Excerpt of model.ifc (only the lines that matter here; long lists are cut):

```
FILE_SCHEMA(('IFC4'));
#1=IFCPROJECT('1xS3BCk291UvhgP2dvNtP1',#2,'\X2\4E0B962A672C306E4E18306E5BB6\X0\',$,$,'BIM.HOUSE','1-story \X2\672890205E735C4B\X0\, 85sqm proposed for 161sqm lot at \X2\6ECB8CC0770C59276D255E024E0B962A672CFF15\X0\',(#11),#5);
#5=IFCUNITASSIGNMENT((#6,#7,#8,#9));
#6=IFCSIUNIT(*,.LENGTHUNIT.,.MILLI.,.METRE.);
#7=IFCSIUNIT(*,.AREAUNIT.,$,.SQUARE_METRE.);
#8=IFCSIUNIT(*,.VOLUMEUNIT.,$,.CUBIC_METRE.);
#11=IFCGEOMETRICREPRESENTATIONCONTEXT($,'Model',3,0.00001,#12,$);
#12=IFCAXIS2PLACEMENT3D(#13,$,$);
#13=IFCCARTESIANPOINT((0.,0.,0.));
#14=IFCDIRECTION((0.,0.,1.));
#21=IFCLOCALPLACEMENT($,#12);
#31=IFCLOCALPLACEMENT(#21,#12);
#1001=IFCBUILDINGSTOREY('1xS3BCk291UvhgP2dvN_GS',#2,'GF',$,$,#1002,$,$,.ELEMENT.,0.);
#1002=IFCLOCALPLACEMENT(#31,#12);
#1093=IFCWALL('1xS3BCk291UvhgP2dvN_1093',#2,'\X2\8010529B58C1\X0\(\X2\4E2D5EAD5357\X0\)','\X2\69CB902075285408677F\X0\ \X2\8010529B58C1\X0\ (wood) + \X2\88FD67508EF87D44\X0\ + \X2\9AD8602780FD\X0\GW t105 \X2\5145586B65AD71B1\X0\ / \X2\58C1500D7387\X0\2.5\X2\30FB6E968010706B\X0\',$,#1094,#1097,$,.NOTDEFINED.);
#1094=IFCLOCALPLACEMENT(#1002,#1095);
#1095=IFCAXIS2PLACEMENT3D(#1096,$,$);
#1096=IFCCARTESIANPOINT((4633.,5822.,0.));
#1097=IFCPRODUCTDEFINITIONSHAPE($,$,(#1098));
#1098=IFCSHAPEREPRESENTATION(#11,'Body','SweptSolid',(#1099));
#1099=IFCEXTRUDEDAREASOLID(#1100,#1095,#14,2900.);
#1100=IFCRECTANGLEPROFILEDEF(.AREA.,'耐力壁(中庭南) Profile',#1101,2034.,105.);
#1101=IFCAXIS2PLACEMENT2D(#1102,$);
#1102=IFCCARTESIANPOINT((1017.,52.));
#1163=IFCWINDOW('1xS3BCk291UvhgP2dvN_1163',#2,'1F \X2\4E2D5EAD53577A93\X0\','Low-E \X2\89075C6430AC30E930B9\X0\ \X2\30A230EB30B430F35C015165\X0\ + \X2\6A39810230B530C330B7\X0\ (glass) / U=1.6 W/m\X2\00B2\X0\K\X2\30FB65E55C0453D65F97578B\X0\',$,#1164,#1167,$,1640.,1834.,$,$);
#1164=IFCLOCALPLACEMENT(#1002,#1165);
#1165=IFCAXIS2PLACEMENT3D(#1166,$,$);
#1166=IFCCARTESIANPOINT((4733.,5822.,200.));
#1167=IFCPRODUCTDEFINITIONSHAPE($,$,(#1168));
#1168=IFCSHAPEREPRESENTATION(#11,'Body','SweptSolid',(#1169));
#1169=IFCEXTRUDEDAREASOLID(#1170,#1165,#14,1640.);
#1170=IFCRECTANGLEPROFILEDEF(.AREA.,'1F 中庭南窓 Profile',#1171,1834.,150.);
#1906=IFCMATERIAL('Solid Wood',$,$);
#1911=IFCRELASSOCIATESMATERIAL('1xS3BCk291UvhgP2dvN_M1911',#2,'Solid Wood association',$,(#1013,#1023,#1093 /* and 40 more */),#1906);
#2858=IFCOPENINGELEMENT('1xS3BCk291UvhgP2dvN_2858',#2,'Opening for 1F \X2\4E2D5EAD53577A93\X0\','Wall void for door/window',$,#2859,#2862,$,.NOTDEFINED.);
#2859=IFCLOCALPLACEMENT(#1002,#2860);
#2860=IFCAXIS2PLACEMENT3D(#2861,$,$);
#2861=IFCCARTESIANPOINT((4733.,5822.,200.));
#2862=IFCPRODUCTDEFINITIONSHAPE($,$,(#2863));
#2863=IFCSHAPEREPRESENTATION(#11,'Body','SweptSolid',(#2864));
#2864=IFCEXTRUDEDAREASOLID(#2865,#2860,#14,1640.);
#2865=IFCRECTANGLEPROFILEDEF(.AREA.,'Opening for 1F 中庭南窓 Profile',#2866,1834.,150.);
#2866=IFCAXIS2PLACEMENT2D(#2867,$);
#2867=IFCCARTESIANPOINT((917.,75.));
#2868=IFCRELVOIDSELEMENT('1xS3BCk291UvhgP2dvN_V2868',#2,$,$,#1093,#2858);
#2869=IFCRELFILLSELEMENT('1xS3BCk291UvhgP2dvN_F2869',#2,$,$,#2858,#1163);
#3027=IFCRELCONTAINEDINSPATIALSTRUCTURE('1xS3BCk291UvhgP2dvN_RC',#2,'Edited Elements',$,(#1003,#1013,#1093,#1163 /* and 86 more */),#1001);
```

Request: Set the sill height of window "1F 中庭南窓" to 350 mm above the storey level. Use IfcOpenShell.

```python
import numpy as np
import ifcopenshell
import ifcopenshell.api.geometry
import ifcopenshell.geom
import ifcopenshell.util.element
import ifcopenshell.util.placement
import ifcopenshell.util.shape
import ifcopenshell.util.unit

model = ifcopenshell.open("model.ifc")
unit_scale = ifcopenshell.util.unit.calculate_unit_scale(model)

window = model.by_id(1163)
opening = window.FillsVoids[0].RelatingOpeningElement
storey = ifcopenshell.util.element.get_container(window, ifc_class="IfcBuildingStorey")
level = ifcopenshell.util.placement.get_local_placement(storey.ObjectPlacement)[2, 3]

# The opening's origin need not be at the sill, so measure its lowest point.
shape = ifcopenshell.geom.create_shape(ifcopenshell.geom.settings(), opening)
bottom = ifcopenshell.util.shape.get_shape_bottom_elevation(shape, shape.geometry) / unit_scale
dz = level + 0.35 / unit_scale - bottom

shift = np.array([0.0, 0.0, dz])
# The window is not placed relative to its opening, so move both.
for product in (opening, window):
    matrix = ifcopenshell.util.placement.get_local_placement(product.ObjectPlacement)
    matrix[:3, 3] += shift
    ifcopenshell.api.geometry.edit_object_placement(model, product=product, matrix=matrix, is_si=False)

print(f"moved by {dz * unit_scale:+.3f} m")

model.write("model_v2.ifc")
```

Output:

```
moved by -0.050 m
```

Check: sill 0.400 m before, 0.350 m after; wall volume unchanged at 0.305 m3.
